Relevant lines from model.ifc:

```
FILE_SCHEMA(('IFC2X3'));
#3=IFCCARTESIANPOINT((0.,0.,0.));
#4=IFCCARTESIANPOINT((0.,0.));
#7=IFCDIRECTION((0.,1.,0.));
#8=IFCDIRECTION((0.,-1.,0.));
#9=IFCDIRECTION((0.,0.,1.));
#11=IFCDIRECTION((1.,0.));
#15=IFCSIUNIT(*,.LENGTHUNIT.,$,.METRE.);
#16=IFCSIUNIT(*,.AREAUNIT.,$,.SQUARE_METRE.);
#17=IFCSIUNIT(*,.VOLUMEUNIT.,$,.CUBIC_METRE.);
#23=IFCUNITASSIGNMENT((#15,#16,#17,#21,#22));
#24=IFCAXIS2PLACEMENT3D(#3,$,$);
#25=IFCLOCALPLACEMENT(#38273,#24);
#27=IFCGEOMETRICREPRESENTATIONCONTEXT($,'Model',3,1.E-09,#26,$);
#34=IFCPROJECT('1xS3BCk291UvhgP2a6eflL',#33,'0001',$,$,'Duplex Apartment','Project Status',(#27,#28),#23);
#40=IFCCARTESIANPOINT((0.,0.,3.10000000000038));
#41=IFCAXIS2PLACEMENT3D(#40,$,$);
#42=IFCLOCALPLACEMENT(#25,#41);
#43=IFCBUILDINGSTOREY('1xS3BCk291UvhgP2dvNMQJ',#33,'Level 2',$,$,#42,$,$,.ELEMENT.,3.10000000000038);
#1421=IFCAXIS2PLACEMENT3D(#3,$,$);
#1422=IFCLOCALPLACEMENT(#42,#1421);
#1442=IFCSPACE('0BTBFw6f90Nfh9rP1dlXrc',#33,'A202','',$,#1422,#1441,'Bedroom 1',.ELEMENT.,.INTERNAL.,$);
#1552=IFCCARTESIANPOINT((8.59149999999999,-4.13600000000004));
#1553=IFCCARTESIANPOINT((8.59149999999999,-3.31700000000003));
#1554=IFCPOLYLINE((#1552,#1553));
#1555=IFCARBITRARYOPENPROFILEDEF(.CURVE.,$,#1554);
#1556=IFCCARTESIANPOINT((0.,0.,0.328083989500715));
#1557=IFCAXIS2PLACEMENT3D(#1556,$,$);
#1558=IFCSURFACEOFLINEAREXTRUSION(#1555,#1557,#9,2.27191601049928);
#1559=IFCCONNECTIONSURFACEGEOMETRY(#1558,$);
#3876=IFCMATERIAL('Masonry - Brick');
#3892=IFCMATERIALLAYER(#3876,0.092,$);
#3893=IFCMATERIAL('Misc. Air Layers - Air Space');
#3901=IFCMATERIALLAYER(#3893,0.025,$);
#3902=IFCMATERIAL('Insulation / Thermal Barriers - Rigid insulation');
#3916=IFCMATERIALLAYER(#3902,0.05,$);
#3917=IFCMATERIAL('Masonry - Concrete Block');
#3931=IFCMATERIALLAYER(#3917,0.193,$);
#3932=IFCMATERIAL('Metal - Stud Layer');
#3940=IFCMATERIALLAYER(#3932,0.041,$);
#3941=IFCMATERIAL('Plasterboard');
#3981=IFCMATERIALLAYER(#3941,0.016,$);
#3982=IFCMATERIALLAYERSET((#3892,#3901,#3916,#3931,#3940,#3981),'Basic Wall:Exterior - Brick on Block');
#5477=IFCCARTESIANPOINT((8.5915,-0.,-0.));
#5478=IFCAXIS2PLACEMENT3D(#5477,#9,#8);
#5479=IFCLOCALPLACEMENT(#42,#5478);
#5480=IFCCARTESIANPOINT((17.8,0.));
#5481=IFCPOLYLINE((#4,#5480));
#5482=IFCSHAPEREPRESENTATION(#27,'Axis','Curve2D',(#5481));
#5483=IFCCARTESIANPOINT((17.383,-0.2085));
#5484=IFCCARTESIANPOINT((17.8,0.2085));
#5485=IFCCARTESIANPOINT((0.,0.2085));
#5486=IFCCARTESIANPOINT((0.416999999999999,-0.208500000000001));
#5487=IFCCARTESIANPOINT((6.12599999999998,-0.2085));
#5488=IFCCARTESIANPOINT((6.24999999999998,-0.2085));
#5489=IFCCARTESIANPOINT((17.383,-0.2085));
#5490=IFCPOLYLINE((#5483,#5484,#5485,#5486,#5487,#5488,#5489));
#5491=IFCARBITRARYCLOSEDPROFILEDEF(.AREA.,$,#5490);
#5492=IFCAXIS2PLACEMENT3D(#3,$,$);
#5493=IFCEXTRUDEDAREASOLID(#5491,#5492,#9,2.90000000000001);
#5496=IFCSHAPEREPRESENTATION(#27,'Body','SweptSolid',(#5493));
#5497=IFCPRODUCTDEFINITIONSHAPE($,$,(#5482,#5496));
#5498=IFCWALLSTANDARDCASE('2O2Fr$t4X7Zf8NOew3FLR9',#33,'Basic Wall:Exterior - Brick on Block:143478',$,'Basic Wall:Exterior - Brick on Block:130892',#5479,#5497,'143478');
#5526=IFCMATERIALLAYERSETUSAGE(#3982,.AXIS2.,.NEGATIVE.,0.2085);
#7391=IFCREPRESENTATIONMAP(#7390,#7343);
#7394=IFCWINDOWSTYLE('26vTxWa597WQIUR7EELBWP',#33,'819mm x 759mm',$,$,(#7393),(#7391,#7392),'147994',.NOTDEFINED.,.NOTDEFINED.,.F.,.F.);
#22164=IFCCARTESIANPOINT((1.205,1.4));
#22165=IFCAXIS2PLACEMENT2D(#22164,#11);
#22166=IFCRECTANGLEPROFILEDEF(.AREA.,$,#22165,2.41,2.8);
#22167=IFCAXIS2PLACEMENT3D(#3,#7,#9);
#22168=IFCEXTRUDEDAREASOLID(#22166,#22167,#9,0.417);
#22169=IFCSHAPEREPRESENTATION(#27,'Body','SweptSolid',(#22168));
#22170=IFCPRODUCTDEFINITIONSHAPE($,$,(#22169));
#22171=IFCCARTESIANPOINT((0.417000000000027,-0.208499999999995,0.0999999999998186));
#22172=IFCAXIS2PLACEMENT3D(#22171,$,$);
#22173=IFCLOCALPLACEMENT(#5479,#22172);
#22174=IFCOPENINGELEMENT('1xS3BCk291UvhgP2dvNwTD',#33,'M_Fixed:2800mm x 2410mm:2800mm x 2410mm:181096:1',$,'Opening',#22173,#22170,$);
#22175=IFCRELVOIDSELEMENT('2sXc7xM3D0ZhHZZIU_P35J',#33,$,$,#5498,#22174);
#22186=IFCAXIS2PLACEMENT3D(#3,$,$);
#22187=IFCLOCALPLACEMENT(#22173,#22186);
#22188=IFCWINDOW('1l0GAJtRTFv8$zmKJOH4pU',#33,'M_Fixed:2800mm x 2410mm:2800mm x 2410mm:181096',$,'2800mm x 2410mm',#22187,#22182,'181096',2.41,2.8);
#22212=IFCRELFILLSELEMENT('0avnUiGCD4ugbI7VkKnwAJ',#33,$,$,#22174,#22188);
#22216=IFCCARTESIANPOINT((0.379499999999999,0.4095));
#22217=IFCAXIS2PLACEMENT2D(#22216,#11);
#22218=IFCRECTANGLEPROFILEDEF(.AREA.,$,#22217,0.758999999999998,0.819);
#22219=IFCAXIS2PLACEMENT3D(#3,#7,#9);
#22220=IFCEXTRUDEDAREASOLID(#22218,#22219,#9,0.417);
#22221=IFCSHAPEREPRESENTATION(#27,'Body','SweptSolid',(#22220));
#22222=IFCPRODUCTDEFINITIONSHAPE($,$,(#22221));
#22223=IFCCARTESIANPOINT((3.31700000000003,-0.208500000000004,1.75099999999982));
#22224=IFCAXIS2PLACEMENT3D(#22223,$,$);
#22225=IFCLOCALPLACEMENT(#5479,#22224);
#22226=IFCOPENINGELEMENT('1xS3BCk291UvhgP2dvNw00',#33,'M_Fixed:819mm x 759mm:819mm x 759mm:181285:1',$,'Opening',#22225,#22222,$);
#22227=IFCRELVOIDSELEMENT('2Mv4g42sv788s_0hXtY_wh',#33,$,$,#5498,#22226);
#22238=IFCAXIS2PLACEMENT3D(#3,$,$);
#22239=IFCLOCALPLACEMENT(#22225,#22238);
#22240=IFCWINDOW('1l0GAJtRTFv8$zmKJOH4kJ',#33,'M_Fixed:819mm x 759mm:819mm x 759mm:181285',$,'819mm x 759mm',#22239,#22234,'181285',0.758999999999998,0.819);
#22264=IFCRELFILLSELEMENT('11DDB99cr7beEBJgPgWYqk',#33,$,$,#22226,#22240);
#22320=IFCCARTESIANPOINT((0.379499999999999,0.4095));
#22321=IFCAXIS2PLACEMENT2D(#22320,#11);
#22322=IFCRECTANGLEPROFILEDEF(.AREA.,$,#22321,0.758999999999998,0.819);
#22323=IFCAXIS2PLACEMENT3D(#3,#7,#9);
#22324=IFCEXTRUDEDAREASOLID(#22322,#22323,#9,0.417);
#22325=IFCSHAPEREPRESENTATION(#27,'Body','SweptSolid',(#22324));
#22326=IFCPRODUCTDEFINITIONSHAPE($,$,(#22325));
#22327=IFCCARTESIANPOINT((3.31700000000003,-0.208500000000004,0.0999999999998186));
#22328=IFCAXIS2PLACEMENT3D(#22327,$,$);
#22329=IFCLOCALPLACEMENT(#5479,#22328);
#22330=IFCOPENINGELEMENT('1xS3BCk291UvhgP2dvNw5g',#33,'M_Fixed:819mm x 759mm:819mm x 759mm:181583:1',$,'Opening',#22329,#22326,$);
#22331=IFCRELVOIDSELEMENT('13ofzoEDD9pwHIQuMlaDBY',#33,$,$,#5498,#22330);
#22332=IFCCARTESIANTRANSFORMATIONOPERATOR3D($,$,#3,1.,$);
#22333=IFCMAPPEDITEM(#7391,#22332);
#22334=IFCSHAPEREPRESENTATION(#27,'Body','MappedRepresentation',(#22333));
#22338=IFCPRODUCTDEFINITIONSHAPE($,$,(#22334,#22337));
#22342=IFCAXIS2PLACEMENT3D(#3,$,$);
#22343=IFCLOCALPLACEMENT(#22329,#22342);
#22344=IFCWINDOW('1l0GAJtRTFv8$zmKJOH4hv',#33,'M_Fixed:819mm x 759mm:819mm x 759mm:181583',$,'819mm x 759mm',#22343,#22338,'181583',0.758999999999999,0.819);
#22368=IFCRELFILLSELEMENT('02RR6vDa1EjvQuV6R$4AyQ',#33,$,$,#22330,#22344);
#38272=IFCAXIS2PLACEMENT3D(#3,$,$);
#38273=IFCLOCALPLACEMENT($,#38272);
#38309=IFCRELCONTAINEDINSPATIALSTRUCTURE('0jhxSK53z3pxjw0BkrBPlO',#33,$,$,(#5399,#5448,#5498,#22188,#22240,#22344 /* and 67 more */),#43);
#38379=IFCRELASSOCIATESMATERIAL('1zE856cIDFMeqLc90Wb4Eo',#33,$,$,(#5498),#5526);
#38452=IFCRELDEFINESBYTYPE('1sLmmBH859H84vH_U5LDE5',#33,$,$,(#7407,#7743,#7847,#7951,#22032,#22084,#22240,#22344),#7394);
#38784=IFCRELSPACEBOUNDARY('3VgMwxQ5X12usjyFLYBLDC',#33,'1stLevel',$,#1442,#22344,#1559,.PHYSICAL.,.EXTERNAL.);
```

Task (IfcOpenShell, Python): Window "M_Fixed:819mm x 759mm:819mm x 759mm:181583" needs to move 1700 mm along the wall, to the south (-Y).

```python
import numpy as np
import ifcopenshell
import ifcopenshell.api.geometry
import ifcopenshell.util.placement
import ifcopenshell.util.unit

model = ifcopenshell.open("model.ifc")
unit_scale = ifcopenshell.util.unit.calculate_unit_scale(model)

window = model.by_guid("1l0GAJtRTFv8$zmKJOH4hv")
opening = window.FillsVoids[0].RelatingOpeningElement
wall = opening.VoidsElements[0].RelatingBuildingElement

wall_matrix = ifcopenshell.util.placement.get_local_placement(wall.ObjectPlacement)
shift = wall_matrix[:3, 0] * 1.7 / unit_scale
before = ifcopenshell.util.placement.get_local_placement(window.ObjectPlacement)[:3, 3].copy()

# The window is placed relative to its opening, so it follows when the opening moves.
matrix = ifcopenshell.util.placement.get_local_placement(opening.ObjectPlacement)
matrix[:3, 3] += shift
ifcopenshell.api.geometry.edit_object_placement(
    model, product=opening, matrix=matrix, is_si=False, should_transform_children=True
)

# Space boundary surfaces are stored in each space's coordinates; move them too.
for rel in window.ProvidesBoundaries:
    if not rel.ConnectionGeometry:
        continue
    surface = rel.ConnectionGeometry.SurfaceOnRelatingElement
    space_matrix = ifcopenshell.util.placement.get_local_placement(rel.RelatingSpace.ObjectPlacement)
    point = np.array(surface.Position.Location.Coordinates) + space_matrix[:3, :3].T @ shift
    surface.Position = model.createIfcAxis2Placement3D(
        model.createIfcCartesianPoint(point.tolist()), surface.Position.Axis, surface.Position.RefDirection
    )

after = ifcopenshell.util.placement.get_local_placement(window.ObjectPlacement)[:3, 3]
print("window moved by", (after - before).round(3) + 0.0)

model.write("model_updated.ifc")
```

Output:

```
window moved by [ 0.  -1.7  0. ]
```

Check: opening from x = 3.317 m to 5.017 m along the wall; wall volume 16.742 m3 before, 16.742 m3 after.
